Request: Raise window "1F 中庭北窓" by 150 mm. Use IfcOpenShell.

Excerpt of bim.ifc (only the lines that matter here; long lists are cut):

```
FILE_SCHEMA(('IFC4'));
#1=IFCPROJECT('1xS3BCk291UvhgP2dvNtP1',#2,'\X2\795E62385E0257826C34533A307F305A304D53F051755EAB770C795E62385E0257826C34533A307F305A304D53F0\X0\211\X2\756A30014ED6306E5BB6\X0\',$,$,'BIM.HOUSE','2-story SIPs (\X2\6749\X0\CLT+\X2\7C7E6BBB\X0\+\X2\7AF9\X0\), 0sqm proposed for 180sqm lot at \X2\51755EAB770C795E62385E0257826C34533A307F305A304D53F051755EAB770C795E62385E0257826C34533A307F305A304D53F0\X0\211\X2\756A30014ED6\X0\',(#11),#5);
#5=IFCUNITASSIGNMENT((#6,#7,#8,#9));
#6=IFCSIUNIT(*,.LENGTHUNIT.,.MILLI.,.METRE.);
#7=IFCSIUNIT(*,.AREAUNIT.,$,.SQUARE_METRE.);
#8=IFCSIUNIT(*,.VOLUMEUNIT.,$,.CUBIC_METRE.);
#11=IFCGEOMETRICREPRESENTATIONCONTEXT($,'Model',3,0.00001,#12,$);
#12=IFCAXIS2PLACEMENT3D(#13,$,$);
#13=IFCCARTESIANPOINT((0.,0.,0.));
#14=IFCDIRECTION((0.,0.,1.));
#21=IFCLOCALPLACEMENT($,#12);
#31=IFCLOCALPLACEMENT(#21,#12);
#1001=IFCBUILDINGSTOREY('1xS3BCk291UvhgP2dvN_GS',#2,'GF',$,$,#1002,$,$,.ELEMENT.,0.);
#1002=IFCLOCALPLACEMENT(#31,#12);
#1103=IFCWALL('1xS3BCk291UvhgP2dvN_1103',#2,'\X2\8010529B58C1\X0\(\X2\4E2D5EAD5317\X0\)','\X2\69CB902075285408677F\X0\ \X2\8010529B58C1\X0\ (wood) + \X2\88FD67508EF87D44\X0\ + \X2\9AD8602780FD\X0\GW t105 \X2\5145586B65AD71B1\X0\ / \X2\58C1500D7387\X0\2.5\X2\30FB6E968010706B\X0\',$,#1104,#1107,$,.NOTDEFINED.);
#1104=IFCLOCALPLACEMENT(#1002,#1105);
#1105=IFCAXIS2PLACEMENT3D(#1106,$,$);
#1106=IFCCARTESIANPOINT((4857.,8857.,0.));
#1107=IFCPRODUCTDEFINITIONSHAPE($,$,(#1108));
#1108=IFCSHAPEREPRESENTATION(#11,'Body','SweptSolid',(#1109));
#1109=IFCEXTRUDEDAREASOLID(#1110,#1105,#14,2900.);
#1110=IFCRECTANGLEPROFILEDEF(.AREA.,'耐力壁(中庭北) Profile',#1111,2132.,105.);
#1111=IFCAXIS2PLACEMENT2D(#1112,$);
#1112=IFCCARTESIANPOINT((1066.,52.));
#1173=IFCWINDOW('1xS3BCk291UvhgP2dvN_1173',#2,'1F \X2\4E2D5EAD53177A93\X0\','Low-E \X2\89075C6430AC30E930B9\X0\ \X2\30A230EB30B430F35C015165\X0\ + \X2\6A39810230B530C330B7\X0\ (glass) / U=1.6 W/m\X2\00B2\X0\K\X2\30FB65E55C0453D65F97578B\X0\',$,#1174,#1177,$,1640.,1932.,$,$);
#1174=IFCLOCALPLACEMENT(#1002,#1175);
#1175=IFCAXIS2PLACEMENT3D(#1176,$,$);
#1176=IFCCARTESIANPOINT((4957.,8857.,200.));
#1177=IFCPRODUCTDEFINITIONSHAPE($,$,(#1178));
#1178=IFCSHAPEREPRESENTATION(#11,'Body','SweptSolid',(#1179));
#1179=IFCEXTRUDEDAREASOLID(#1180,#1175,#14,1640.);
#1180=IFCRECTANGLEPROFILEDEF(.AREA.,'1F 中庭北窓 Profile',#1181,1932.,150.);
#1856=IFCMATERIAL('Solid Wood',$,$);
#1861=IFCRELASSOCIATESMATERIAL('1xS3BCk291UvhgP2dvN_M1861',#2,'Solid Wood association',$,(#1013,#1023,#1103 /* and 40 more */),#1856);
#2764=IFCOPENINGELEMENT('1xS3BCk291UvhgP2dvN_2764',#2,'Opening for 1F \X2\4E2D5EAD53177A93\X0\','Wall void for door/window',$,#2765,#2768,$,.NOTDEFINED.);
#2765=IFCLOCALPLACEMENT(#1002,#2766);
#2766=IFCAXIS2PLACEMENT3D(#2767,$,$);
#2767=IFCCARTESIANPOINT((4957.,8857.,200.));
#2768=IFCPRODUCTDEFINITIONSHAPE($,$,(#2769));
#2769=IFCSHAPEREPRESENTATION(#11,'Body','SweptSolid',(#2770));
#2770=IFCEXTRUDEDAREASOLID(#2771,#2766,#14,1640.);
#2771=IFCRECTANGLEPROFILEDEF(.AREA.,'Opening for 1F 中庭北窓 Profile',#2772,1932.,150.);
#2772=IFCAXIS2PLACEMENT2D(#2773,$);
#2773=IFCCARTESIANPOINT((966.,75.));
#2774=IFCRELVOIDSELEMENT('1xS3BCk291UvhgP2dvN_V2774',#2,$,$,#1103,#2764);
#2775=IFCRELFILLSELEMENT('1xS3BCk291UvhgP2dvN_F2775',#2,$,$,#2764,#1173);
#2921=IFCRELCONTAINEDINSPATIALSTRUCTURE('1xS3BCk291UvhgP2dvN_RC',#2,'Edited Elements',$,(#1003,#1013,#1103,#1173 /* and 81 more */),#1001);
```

```python
import numpy as np
import ifcopenshell
import ifcopenshell.api.geometry
import ifcopenshell.util.placement
import ifcopenshell.util.unit

model = ifcopenshell.open("bim.ifc")
unit_scale = ifcopenshell.util.unit.calculate_unit_scale(model)

window = model.by_guid("1xS3BCk291UvhgP2dvN_1173")
opening = window.FillsVoids[0].RelatingOpeningElement
dz = 0.15 / unit_scale

shift = np.array([0.0, 0.0, dz])
# The window is not placed relative to its opening, so move both.
for product in (opening, window):
    matrix = ifcopenshell.util.placement.get_local_placement(product.ObjectPlacement)
    matrix[:3, 3] += shift
    ifcopenshell.api.geometry.edit_object_placement(model, product=product, matrix=matrix, is_si=False)

print(f"moved by {dz * unit_scale:+.3f} m")

model.write("bim_updated.ifc")
```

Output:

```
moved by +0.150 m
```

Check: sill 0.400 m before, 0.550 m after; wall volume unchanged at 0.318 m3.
